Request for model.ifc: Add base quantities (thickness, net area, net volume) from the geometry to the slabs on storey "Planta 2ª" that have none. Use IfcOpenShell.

First a look at what the model holds.

```python
import ifcopenshell
import ifcopenshell.util.element
import ifcopenshell.util.unit

model = ifcopenshell.open("model.ifc")
print(model.schema)
for unit_type in ("LENGTHUNIT", "AREAUNIT", "VOLUMEUNIT"):
    print(unit_type, ifcopenshell.util.unit.calculate_unit_scale(model, unit_type))
storey = next(s for s in model.by_type("IfcBuildingStorey") if s.Name == "Planta 2ª")
slabs = [e for e in ifcopenshell.util.element.get_decomposition(storey) if e.is_a("IfcSlab")]
for e in sorted(slabs, key=lambda e: e.id()):
    print(e.id(), e.is_a(), e.Name, list(ifcopenshell.util.element.get_psets(e, qtos_only=True)), sep=" | ")
```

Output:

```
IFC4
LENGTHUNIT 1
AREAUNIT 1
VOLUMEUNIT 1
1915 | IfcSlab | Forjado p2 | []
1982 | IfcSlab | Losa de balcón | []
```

```python
import ifcopenshell
import ifcopenshell.api.pset
import ifcopenshell.geom
import ifcopenshell.util.element
import ifcopenshell.util.shape
import ifcopenshell.util.unit

model = ifcopenshell.open("model.ifc")
unit_scale = ifcopenshell.util.unit.calculate_unit_scale(model)
area_scale = ifcopenshell.util.unit.calculate_unit_scale(model, "AREAUNIT")
volume_scale = ifcopenshell.util.unit.calculate_unit_scale(model, "VOLUMEUNIT")
settings = ifcopenshell.geom.settings()

storey = next(s for s in model.by_type("IfcBuildingStorey") if s.Name == "Planta 2ª")
slabs = [e for e in ifcopenshell.util.element.get_decomposition(storey) if e.is_a("IfcSlab")]

for e in sorted(slabs, key=lambda e: e.id()):
    if ifcopenshell.util.element.get_psets(e, qtos_only=True, should_inherit=False):
        continue
    # Geometry comes back in metres, in the element's own axes.
    shape = ifcopenshell.geom.create_shape(settings, e)
    values = {
        "Width": ifcopenshell.util.shape.get_z(shape.geometry) / unit_scale,
        "NetArea": ifcopenshell.util.shape.get_footprint_area(shape.geometry) / area_scale,
        "NetVolume": ifcopenshell.util.shape.get_volume(shape.geometry) / volume_scale,
    }
    qto = ifcopenshell.api.pset.add_qto(model, product=e, name="Qto_SlabBaseQuantities")
    ifcopenshell.api.pset.edit_qto(model, qto=qto, properties=values)
    print(e.id(), {k: round(v, 3) for k, v in values.items()})

model.write("model-out.ifc")
```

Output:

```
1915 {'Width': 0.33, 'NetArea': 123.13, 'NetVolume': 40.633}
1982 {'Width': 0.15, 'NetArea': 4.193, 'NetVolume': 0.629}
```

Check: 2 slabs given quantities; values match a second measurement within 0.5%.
